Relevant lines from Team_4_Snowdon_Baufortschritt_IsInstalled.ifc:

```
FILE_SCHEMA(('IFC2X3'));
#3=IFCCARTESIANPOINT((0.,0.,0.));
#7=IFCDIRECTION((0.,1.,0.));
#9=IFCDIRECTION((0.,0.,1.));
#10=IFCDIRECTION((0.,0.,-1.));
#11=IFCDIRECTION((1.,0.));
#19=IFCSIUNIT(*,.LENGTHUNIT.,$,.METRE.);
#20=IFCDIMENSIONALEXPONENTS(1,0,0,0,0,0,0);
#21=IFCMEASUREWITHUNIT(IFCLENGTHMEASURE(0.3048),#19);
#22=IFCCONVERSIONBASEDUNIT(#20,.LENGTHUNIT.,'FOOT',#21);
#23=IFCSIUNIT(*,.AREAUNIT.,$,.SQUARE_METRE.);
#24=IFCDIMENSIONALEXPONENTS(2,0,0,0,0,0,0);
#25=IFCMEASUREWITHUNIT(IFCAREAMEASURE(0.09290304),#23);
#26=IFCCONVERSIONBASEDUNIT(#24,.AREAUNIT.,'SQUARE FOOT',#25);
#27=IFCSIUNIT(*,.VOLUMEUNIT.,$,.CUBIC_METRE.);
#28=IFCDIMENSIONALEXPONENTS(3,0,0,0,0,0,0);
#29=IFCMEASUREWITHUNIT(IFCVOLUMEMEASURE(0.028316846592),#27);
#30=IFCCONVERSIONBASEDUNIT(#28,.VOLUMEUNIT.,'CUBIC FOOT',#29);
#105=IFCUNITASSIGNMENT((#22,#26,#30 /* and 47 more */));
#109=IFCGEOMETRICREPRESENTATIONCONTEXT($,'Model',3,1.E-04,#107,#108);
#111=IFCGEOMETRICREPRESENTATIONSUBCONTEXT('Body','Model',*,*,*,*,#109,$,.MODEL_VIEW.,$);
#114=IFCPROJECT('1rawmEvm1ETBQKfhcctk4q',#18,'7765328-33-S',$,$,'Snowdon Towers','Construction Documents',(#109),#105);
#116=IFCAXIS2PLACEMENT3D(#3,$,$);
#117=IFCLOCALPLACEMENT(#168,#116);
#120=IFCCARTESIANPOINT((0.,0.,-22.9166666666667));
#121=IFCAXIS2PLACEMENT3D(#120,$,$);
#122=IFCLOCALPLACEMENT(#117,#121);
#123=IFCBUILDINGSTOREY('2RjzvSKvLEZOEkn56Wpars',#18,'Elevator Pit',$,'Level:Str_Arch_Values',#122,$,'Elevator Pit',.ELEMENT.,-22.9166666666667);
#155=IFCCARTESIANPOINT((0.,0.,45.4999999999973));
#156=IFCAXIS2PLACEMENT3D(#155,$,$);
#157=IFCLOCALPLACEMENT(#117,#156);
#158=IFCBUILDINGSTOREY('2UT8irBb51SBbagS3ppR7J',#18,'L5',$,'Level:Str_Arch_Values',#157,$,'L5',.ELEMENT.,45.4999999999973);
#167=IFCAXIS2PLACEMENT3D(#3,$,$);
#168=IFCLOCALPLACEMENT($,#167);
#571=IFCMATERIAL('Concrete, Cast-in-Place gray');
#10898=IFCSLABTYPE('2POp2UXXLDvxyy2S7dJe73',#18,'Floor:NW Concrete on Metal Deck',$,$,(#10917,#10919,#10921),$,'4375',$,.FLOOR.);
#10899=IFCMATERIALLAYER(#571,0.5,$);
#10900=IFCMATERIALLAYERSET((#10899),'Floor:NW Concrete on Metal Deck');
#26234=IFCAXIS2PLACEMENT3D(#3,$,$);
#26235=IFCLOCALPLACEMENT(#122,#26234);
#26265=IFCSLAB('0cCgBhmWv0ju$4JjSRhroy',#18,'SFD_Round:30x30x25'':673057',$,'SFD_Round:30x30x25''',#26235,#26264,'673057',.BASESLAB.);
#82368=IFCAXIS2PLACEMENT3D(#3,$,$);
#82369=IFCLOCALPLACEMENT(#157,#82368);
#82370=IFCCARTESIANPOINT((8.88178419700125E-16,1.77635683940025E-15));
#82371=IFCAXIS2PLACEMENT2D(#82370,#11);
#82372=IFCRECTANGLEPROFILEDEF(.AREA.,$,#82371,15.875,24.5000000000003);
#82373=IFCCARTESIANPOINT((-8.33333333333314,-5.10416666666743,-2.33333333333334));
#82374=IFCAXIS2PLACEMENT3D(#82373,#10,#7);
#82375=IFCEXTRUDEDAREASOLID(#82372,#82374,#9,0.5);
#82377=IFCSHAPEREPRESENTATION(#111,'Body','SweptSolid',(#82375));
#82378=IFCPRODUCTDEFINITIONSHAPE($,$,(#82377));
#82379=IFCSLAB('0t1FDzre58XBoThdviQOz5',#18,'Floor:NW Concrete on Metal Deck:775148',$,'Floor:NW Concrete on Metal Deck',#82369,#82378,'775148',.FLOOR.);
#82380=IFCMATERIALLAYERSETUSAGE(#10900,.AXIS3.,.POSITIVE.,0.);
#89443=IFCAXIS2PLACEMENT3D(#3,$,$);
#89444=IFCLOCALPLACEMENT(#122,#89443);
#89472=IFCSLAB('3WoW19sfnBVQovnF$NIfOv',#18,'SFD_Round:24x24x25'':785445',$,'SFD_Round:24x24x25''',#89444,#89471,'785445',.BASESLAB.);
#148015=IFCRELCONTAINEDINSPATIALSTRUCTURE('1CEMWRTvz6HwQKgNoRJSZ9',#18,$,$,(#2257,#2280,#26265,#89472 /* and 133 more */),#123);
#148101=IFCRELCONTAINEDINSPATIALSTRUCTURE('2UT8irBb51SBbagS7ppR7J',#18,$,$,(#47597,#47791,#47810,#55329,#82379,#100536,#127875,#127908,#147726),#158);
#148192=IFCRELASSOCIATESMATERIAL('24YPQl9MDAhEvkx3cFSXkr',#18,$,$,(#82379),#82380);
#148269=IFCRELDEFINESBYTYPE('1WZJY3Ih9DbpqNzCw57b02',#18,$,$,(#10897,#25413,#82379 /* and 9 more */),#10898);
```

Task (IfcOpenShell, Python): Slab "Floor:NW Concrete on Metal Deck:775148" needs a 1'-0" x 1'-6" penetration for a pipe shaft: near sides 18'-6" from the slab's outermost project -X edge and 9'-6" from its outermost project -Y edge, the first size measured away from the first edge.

```python
import numpy as np
import ifcopenshell
import ifcopenshell.api.feature
import ifcopenshell.api.geometry
import ifcopenshell.api.root
import ifcopenshell.geom
import ifcopenshell.util.placement
import ifcopenshell.util.representation
import ifcopenshell.util.shape
import ifcopenshell.util.unit

model = ifcopenshell.open("Team_4_Snowdon_Baufortschritt_IsInstalled.ifc")
unit_scale = ifcopenshell.util.unit.calculate_unit_scale(model)
settings = ifcopenshell.geom.settings()


def volume(element):
    """Net volume in cubic metres, openings subtracted."""
    shape = ifcopenshell.geom.create_shape(settings, element)
    return ifcopenshell.util.shape.get_volume(shape.geometry)


slab = model.by_guid("0t1FDzre58XBoThdviQOz5")
before = volume(slab)

# Extent in the slab's own axes, in metres. The edges named are its -X and -Y sides.
slab_shape = ifcopenshell.geom.create_shape(settings, slab)
vertices = ifcopenshell.util.shape.get_vertices(slab_shape.geometry)
x_min, y_min, bottom = vertices.min(axis=0)
top = vertices[:, 2].max()

opening = ifcopenshell.api.root.create_entity(model, ifc_class="IfcOpeningElement", name="Pipe shaft opening")
context = ifcopenshell.util.representation.get_context(model, "Model", "Body", "MODEL_VIEW")
width, depth = 0.3048, 0.4572
outline = [(0.0, 0.0), (width, 0.0), (width, depth), (0.0, depth), (0.0, 0.0)]
# Overshoot both faces by 50 mm so the cut is clean.
shape = ifcopenshell.api.geometry.add_slab_representation(
    model, context=context, depth=top - bottom + 0.1, polyline=outline
)
ifcopenshell.api.geometry.assign_representation(model, product=opening, representation=shape)

matrix = ifcopenshell.util.placement.get_local_placement(slab.ObjectPlacement)
matrix[:, 3] = matrix @ np.append(np.array([x_min + 5.6388, y_min + 2.8956, bottom - 0.05]) / unit_scale, 1.0)
ifcopenshell.api.geometry.edit_object_placement(model, product=opening, matrix=matrix, is_si=False)
ifcopenshell.api.feature.add_feature(model, feature=opening, element=slab)

after = volume(slab)

print(f"slab volume {before:.3f} -> {after:.3f} m3")

model.write("Team_4_Snowdon_Baufortschritt_IsInstalled_edited.ifc")
```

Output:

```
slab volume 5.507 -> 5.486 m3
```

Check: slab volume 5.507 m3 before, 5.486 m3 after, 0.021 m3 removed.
